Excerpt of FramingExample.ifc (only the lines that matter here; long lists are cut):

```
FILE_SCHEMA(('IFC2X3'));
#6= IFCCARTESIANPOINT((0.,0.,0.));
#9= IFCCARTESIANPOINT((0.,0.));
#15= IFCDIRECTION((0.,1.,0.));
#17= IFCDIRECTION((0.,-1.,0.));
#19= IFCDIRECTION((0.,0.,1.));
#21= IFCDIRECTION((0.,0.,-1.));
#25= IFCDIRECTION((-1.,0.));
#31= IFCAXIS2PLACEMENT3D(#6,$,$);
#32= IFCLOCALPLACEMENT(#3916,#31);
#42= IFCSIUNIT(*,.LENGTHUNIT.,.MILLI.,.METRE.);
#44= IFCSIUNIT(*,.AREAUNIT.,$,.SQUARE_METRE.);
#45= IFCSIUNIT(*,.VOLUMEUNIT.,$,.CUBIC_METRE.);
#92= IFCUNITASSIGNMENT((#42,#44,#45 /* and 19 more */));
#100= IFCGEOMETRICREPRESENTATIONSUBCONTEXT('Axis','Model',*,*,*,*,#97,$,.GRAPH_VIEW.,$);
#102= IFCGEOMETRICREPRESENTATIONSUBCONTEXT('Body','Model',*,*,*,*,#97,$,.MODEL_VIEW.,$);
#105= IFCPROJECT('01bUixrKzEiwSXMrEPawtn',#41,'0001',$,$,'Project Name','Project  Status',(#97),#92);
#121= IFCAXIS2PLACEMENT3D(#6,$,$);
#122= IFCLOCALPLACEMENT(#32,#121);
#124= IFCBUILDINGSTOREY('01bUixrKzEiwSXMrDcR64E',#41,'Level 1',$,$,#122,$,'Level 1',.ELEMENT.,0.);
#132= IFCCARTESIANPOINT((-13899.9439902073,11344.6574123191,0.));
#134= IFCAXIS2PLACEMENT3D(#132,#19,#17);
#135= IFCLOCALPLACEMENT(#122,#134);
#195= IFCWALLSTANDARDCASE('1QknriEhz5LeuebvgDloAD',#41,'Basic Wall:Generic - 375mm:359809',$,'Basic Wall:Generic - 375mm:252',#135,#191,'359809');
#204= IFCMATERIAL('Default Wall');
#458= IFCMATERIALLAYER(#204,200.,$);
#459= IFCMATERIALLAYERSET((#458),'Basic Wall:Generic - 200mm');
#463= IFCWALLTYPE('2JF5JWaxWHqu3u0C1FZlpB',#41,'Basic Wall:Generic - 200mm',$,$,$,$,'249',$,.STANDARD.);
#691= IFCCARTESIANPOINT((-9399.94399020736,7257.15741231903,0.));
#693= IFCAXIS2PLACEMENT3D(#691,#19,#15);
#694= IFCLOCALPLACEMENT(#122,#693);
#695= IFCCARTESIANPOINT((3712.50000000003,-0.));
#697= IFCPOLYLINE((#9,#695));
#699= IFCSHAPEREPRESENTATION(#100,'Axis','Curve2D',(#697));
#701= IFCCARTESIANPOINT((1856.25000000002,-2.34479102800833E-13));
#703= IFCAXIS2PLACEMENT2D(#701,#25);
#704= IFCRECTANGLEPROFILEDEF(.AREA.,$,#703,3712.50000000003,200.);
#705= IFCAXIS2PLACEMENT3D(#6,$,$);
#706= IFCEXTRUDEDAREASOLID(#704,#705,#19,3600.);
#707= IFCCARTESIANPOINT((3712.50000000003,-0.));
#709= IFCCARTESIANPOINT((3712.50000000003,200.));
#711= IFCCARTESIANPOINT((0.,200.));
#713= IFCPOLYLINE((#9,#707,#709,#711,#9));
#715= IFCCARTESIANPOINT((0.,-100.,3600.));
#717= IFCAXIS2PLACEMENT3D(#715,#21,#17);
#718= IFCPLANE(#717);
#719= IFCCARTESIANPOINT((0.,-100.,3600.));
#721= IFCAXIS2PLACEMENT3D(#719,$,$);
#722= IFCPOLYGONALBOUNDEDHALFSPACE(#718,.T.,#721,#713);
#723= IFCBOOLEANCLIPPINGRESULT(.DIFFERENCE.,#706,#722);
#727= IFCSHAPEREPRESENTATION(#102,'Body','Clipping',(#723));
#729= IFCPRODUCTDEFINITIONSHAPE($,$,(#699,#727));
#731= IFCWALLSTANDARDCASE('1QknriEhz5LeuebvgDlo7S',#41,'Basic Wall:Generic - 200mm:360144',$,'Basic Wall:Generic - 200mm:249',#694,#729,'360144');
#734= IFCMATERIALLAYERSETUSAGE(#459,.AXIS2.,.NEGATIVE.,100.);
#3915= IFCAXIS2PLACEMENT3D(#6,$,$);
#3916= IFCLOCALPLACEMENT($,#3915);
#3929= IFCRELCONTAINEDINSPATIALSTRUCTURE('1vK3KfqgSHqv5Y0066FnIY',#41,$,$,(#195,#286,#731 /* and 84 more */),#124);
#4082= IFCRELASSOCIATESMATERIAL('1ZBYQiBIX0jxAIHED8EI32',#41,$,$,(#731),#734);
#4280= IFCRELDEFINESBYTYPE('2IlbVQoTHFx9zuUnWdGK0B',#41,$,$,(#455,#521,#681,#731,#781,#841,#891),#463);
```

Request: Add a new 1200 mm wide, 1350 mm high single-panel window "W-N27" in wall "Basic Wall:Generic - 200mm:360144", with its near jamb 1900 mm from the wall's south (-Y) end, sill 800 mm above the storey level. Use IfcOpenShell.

```python
import numpy as np
import ifcopenshell
import ifcopenshell.api.feature
import ifcopenshell.api.geometry
import ifcopenshell.api.root
import ifcopenshell.api.spatial
import ifcopenshell.api.type
import ifcopenshell.geom
import ifcopenshell.util.element
import ifcopenshell.util.placement
import ifcopenshell.util.representation
import ifcopenshell.util.shape
import ifcopenshell.util.unit

model = ifcopenshell.open("FramingExample.ifc")
unit_scale = ifcopenshell.util.unit.calculate_unit_scale(model)
settings = ifcopenshell.geom.settings()


def volume(element):
    """Net volume in cubic metres, openings subtracted."""
    shape = ifcopenshell.geom.create_shape(settings, element)
    return ifcopenshell.util.shape.get_volume(shape.geometry)


wall = model.by_guid("1QknriEhz5LeuebvgDlo7S")
storey = ifcopenshell.util.element.get_container(wall, ifc_class="IfcBuildingStorey")
context = ifcopenshell.util.representation.get_context(model, "Model", "Body", "MODEL_VIEW")
before = volume(wall)

width, height, from_end, sill = 1.2, 1.35, 1.9, 0.8  # metres

# The wall runs along its own X axis, and the end named is its -X end.
wall_shape = ifcopenshell.geom.create_shape(settings, wall)
x, y, z = ifcopenshell.util.shape.get_vertices(wall_shape.geometry).T
start = x.min() + from_end
face, thickness = float(y.min()), float(y.max() - y.min())
wall_matrix = ifcopenshell.util.placement.get_local_placement(wall.ObjectPlacement)
level = ifcopenshell.util.placement.get_local_placement(storey.ObjectPlacement)[2, 3]


def in_wall(x, y):
    """Placement at x, y metres in the wall's axes, at sill height."""
    matrix = wall_matrix.copy()
    matrix[:, 3] = wall_matrix @ np.array([x / unit_scale, y / unit_scale, 0.0, 1.0])
    matrix[2, 3] = level + sill / unit_scale
    return matrix


# Opening: a box that overshoots both wall faces by 50 mm.
opening = ifcopenshell.api.root.create_entity(model, ifc_class="IfcOpeningElement")
box = ifcopenshell.api.geometry.add_wall_representation(
    model, context=context, length=width, height=height, thickness=thickness + 0.1
)
ifcopenshell.api.geometry.assign_representation(model, product=opening, representation=box)
ifcopenshell.api.geometry.edit_object_placement(model, product=opening, matrix=in_wall(start, face - 0.05), is_si=False)
ifcopenshell.api.feature.add_feature(model, feature=opening, element=wall)

window = ifcopenshell.api.root.create_entity(model, ifc_class="IfcWindow", name="W-N27")
window.OverallWidth, window.OverallHeight = width / unit_scale, height / unit_scale
body = ifcopenshell.api.geometry.add_window_representation(
    model,
    context=context,
    overall_width=window.OverallWidth,
    overall_height=window.OverallHeight,
    partition_type="SINGLE_PANEL",
)
ifcopenshell.api.geometry.assign_representation(model, product=window, representation=body)
ifcopenshell.api.spatial.assign_container(model, products=[window], relating_structure=storey)
fills = ifcopenshell.api.feature.add_filling(model, opening=opening, element=window)
fills.OwnerHistory = window.OwnerHistory  # required in IFC2X3

# IFC2X3 keeps the operation on the window style.
style = ifcopenshell.api.root.create_entity(model, ifc_class="IfcWindowStyle", name="W-N27")
style.OperationType, style.ConstructionType = "SINGLE_PANEL", "NOTDEFINED"
style.ParameterTakesPrecedence = style.Sizeable = False
ifcopenshell.api.type.assign_type(model, related_objects=[window], relating_type=style)

# Centre the window in the wall's thickness.
ifcopenshell.api.geometry.edit_object_placement(model, product=window, matrix=in_wall(start, face), is_si=False)
window_shape = ifcopenshell.geom.create_shape(settings, window)
depth = ifcopenshell.util.shape.get_vertices(window_shape.geometry)[:, 1]
offset = face + thickness / 2 - (depth.min() + depth.max()) / 2
ifcopenshell.api.geometry.edit_object_placement(model, product=window, matrix=in_wall(start, offset), is_si=False)

after = volume(wall)

print(f"wall volume {before:.3f} -> {after:.3f} m3")

model.write("FramingExample_rev.ifc")
```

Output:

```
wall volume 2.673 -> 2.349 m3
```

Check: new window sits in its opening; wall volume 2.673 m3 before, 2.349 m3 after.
